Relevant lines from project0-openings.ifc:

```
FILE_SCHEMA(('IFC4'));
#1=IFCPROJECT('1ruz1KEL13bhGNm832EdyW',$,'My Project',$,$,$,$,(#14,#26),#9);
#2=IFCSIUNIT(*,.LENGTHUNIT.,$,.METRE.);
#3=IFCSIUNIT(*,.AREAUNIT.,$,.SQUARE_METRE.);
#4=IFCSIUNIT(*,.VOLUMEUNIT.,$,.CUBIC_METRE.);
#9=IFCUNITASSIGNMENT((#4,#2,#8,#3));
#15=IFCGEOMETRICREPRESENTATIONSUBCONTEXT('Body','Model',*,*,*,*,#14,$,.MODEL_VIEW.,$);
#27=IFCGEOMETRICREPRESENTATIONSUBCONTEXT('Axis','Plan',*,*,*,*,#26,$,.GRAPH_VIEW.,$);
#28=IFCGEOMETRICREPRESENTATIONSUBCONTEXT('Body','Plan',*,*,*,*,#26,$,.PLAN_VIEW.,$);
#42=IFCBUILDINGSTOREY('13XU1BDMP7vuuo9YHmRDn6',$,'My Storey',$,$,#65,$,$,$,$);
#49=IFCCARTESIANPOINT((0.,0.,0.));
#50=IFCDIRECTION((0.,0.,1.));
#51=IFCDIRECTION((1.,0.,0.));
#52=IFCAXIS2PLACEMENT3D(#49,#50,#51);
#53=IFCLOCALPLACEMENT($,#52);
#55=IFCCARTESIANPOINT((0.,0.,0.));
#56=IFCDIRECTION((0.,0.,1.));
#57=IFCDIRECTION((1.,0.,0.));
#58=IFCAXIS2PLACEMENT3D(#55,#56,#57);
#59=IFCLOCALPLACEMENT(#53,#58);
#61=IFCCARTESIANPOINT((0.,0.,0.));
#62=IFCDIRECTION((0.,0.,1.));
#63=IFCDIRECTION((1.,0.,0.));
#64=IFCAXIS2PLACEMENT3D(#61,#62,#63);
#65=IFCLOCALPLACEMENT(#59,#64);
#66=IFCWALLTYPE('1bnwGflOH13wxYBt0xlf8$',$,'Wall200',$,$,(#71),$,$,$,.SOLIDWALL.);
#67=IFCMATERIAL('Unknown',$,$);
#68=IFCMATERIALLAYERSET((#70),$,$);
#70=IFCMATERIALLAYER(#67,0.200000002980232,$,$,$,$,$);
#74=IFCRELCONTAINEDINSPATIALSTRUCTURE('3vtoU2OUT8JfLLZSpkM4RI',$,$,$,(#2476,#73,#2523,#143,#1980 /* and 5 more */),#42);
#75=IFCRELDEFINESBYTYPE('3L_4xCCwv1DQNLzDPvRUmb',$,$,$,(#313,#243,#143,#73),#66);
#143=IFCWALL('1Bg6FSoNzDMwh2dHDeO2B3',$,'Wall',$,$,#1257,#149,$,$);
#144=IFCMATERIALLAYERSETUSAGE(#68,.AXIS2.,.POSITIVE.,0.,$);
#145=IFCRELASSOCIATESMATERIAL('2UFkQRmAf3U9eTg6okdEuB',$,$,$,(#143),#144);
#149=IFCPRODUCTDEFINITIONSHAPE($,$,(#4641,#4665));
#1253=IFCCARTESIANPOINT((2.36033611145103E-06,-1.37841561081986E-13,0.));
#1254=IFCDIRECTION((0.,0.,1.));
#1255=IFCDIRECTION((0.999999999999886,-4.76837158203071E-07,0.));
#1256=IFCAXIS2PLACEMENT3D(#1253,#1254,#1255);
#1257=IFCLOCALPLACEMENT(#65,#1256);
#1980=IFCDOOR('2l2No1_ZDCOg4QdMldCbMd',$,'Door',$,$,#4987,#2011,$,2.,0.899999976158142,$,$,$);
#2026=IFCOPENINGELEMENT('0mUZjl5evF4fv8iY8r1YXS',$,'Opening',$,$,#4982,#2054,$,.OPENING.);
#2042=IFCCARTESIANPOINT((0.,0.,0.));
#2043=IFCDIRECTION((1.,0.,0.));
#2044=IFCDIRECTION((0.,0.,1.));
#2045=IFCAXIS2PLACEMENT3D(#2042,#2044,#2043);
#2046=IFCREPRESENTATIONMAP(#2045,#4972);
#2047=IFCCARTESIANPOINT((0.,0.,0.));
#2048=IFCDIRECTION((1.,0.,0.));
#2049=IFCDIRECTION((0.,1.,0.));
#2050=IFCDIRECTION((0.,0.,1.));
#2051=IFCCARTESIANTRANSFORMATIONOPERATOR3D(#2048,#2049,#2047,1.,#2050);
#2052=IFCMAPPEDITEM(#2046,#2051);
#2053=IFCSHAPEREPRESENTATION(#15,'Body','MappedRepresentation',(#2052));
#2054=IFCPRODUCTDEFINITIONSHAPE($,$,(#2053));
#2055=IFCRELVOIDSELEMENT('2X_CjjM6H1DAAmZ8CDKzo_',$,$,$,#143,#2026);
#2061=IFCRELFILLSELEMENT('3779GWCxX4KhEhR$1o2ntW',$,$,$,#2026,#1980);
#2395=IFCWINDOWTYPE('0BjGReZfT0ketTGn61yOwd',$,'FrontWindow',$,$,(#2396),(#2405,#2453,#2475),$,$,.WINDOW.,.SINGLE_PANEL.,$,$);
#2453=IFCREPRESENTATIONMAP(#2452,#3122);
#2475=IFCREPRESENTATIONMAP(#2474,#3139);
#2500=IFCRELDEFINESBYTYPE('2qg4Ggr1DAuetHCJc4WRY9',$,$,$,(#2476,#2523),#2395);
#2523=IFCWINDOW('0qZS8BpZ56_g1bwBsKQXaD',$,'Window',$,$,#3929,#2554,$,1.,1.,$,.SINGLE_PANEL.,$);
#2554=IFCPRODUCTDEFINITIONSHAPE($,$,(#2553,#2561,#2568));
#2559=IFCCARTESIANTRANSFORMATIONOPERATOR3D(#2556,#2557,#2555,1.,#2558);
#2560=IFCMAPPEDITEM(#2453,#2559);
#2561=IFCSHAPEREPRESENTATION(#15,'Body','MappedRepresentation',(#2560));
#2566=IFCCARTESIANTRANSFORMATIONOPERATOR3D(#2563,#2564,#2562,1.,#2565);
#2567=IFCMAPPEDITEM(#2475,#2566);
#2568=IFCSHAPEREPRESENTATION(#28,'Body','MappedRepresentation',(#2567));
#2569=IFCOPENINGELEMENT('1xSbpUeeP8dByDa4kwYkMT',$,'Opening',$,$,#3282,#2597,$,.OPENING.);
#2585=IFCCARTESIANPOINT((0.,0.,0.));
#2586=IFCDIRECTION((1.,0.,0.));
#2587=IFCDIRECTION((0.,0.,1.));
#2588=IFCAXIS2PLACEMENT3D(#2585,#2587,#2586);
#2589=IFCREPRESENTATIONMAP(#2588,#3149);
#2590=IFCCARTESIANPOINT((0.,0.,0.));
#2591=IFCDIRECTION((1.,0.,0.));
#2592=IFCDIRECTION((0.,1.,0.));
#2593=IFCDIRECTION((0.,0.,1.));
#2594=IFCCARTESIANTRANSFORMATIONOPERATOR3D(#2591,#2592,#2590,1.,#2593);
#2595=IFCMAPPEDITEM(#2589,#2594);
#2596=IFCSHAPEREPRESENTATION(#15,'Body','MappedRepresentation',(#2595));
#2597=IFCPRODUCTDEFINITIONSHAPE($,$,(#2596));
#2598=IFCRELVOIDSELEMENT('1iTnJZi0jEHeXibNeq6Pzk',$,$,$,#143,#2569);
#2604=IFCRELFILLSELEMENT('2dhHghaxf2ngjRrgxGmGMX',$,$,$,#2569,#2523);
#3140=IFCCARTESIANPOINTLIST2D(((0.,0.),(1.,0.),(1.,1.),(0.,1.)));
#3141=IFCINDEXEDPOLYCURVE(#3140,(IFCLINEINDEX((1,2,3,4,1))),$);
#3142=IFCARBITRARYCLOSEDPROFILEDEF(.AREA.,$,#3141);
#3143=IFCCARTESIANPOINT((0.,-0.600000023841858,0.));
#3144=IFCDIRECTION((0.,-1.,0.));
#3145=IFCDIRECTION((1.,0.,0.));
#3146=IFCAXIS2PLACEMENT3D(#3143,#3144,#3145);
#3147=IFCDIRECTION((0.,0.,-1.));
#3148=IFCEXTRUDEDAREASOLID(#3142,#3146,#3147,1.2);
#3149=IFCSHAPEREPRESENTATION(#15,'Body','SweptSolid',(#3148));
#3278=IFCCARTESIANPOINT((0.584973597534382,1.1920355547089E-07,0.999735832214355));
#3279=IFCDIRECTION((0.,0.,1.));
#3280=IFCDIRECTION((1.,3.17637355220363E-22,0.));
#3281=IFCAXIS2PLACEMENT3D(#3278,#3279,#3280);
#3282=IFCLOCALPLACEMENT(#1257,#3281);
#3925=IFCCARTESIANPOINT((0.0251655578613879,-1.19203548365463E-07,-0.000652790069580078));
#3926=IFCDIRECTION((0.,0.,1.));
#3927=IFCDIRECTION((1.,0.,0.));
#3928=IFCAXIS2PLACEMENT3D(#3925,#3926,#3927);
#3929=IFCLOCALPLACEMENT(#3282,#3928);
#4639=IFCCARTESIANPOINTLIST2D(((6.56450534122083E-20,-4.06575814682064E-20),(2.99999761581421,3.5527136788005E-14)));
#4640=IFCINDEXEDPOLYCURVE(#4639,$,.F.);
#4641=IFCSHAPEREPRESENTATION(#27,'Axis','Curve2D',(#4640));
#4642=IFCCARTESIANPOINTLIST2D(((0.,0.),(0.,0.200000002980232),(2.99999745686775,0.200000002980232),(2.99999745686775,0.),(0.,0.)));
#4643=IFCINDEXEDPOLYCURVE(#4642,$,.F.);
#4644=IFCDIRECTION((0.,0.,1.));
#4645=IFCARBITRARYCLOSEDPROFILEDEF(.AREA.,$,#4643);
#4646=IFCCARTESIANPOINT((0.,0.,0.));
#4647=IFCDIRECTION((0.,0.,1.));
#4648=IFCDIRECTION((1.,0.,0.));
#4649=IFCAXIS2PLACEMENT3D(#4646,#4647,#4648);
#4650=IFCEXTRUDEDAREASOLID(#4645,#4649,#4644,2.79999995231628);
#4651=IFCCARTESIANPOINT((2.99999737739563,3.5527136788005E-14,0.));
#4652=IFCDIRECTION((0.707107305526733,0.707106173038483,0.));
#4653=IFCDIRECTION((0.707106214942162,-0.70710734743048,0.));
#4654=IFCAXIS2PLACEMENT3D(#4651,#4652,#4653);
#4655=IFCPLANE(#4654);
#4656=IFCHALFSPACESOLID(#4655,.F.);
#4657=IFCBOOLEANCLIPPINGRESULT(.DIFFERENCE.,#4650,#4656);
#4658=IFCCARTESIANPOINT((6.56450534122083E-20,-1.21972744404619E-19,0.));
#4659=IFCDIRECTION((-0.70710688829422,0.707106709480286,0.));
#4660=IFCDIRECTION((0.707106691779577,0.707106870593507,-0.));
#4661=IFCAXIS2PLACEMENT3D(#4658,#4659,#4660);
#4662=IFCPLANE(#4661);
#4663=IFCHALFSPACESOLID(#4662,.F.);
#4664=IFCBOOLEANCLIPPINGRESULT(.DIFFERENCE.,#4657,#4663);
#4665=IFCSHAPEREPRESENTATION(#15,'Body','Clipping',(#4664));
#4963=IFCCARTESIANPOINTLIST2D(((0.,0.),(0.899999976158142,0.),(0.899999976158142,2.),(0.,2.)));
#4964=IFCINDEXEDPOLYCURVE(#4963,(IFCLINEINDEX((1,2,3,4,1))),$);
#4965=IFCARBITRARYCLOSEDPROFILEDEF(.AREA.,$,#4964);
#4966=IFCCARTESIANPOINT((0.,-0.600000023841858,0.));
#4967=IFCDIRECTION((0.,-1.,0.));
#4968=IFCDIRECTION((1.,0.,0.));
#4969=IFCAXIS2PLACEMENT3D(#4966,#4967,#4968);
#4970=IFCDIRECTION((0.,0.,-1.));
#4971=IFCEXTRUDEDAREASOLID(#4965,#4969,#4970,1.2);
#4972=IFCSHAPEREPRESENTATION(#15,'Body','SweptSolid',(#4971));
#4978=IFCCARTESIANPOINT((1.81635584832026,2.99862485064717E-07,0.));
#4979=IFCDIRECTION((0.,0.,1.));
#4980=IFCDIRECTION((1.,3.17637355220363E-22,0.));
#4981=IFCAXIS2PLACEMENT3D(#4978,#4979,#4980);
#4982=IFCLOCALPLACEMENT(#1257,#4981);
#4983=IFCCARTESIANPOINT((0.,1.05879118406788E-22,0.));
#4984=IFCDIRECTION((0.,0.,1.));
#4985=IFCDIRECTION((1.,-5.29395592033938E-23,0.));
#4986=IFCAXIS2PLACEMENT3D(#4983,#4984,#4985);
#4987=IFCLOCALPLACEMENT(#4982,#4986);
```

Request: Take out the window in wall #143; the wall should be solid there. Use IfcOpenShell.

```python
import ifcopenshell
import ifcopenshell.api.feature
import ifcopenshell.api.root
import ifcopenshell.geom
import ifcopenshell.util.shape

model = ifcopenshell.open("project0-openings.ifc")
settings = ifcopenshell.geom.settings()


def volume(element):
    """Net volume in cubic metres, openings subtracted."""
    shape = ifcopenshell.geom.create_shape(settings, element)
    return ifcopenshell.util.shape.get_volume(shape.geometry)


window = model.by_guid("0qZS8BpZ56_g1bwBsKQXaD")
opening = window.FillsVoids[0].RelatingOpeningElement
wall = opening.VoidsElements[0].RelatingBuildingElement
before = volume(wall)

ifcopenshell.api.root.remove_product(model, product=window)
ifcopenshell.api.feature.remove_feature(model, feature=opening)

after = volume(wall)

print(f"wall volume {before:.3f} -> {after:.3f} m3")

model.write("project0-openings_edited.ifc")
```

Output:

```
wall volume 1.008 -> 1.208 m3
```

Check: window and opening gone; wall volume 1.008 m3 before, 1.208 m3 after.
